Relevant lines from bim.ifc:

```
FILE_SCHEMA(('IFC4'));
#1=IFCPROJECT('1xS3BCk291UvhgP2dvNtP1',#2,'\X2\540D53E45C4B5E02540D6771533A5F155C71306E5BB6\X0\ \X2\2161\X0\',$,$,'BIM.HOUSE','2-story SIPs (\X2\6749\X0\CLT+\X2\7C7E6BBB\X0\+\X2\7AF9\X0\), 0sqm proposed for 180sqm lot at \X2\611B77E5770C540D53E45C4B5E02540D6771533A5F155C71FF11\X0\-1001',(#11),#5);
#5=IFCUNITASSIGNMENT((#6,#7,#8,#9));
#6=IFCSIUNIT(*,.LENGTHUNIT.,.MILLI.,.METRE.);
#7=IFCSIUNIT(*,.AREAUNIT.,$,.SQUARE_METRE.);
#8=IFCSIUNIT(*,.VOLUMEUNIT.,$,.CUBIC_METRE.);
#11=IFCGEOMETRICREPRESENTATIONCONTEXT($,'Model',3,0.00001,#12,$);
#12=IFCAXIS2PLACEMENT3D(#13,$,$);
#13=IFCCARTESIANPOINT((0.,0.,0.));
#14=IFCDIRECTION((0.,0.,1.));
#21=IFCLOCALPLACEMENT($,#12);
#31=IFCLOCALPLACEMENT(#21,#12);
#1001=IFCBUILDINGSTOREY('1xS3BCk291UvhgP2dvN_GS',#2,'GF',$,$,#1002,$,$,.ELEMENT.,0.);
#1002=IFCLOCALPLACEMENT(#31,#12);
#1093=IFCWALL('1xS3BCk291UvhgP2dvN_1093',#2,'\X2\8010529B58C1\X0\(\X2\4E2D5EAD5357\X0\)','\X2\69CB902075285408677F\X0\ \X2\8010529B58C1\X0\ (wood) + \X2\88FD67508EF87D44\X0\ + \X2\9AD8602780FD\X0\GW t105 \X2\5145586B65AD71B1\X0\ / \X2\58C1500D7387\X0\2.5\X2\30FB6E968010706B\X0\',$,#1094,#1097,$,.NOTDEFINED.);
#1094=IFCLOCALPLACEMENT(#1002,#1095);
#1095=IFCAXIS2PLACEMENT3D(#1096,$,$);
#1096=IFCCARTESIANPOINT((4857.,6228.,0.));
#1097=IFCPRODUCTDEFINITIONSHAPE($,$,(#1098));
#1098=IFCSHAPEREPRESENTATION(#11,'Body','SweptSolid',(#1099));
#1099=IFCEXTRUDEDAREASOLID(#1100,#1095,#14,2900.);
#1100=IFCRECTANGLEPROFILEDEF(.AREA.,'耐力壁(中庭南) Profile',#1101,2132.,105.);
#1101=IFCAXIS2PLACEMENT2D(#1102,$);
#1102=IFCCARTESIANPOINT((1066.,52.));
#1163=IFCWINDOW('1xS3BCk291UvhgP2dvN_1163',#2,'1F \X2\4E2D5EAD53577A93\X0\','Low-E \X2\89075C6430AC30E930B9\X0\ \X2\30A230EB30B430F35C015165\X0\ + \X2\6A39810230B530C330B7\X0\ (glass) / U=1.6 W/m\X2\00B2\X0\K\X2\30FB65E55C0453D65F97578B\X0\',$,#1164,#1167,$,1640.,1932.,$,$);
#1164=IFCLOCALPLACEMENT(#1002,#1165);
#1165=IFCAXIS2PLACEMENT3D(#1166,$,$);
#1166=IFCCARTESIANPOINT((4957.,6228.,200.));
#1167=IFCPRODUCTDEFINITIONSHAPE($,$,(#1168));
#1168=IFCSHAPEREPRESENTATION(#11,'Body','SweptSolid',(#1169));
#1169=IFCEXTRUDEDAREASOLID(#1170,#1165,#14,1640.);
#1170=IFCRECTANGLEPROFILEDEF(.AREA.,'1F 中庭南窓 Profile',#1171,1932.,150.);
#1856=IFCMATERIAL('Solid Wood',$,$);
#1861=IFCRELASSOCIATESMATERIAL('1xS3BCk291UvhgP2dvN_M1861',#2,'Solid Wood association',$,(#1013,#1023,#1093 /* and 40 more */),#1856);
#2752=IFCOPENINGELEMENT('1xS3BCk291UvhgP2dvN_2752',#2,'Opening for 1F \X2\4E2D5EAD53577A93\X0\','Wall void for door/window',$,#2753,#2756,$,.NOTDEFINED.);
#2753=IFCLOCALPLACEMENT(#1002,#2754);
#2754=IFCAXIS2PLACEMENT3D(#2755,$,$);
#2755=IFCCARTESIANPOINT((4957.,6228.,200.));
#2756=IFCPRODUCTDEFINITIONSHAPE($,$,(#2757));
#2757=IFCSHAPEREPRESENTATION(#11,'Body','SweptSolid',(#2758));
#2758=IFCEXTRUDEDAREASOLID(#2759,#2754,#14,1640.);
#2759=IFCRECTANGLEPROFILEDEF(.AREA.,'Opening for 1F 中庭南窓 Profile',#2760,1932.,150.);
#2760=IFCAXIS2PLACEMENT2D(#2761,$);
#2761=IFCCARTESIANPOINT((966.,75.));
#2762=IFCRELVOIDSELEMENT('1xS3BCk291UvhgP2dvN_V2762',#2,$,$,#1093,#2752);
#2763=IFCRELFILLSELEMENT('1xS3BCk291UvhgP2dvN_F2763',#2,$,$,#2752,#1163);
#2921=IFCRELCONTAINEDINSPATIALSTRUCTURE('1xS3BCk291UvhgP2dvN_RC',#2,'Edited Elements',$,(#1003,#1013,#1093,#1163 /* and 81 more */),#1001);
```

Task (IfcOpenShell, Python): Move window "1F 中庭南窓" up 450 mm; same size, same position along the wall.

```python
import numpy as np
import ifcopenshell
import ifcopenshell.api.geometry
import ifcopenshell.util.placement
import ifcopenshell.util.unit

model = ifcopenshell.open("bim.ifc")
unit_scale = ifcopenshell.util.unit.calculate_unit_scale(model)

window = model.by_guid("1xS3BCk291UvhgP2dvN_1163")
opening = window.FillsVoids[0].RelatingOpeningElement
dz = 0.45 / unit_scale

shift = np.array([0.0, 0.0, dz])
# The window is not placed relative to its opening, so move both.
for product in (opening, window):
    matrix = ifcopenshell.util.placement.get_local_placement(product.ObjectPlacement)
    matrix[:3, 3] += shift
    ifcopenshell.api.geometry.edit_object_placement(model, product=product, matrix=matrix, is_si=False)

print(f"moved by {dz * unit_scale:+.3f} m")

model.write("bim-out.ifc")
```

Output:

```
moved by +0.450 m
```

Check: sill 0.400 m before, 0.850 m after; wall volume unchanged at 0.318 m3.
